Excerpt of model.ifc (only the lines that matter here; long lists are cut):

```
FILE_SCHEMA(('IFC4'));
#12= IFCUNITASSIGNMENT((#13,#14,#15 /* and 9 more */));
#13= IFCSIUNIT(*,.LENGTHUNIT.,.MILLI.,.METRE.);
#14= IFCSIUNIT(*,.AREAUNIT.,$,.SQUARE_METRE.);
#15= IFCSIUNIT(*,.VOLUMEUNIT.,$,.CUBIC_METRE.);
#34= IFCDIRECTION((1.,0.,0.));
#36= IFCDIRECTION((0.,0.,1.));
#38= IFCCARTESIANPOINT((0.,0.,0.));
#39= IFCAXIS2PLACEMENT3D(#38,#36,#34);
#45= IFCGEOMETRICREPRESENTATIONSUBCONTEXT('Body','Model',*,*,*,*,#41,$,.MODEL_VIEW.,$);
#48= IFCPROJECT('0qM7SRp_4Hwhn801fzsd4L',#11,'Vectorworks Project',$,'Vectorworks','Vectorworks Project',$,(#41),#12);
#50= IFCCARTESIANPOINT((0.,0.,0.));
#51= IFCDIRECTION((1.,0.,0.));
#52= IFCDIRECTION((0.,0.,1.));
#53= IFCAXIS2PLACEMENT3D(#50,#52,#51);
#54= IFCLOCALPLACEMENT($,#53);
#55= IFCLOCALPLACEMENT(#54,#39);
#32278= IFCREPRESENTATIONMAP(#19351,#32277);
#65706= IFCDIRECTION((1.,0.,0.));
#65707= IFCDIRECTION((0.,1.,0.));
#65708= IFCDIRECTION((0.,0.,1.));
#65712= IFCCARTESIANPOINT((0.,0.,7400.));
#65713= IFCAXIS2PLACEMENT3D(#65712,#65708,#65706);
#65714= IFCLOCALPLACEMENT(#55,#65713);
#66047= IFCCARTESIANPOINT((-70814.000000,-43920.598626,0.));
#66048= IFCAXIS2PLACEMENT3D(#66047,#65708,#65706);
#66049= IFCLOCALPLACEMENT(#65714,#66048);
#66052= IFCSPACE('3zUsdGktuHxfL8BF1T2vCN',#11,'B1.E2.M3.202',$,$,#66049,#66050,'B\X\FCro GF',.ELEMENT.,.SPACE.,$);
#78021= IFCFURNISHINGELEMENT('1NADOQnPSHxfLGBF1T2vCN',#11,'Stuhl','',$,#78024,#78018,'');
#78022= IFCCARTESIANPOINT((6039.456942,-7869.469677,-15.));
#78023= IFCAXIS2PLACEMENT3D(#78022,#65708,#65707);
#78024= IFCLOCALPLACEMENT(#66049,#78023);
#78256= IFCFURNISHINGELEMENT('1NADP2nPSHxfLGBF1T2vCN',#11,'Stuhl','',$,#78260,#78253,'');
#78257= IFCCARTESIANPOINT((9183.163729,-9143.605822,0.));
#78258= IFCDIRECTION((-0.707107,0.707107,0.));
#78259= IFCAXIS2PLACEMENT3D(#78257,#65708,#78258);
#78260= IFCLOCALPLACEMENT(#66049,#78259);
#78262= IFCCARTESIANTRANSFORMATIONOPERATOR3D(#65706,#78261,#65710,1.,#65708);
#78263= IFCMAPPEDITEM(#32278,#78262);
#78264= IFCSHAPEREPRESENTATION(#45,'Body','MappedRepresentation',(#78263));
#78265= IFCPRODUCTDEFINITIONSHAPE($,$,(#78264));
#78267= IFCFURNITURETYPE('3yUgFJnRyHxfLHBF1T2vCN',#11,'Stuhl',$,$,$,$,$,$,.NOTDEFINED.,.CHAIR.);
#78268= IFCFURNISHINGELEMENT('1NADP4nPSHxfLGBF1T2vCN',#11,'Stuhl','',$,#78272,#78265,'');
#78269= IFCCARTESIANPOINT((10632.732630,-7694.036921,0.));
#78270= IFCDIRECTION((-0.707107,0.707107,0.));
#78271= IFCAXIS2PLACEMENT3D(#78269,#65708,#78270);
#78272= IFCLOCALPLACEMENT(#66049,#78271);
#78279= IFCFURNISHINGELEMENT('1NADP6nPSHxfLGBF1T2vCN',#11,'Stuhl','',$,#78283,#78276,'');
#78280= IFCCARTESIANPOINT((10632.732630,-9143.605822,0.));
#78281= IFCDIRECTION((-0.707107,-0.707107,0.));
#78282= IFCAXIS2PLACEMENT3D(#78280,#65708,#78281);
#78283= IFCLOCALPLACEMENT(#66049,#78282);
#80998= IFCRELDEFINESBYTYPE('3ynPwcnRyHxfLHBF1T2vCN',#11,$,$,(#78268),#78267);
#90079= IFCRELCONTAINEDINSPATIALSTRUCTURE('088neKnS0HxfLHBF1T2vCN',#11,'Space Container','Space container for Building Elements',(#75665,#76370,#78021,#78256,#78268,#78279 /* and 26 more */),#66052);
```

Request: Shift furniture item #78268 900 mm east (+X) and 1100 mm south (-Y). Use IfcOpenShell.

```python
import ifcopenshell
import ifcopenshell.api.geometry
import ifcopenshell.util.placement

model = ifcopenshell.open("model.ifc")

item = model.by_guid("1NADP4nPSHxfLGBF1T2vCN")
matrix = ifcopenshell.util.placement.get_local_placement(item.ObjectPlacement)
matrix[0, 3] += 900.0
matrix[1, 3] -= 1100.0
ifcopenshell.api.geometry.edit_object_placement(model, product=item, matrix=matrix, is_si=False)

print(ifcopenshell.util.placement.get_local_placement(item.ObjectPlacement).round(3) + 0.0)

model.write("model_v2.ifc")
```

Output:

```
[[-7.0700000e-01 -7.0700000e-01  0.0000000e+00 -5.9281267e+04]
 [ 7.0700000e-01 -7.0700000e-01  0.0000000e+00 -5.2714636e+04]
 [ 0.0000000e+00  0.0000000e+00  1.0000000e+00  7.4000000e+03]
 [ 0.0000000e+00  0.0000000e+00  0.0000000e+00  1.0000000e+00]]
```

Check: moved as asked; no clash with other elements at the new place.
